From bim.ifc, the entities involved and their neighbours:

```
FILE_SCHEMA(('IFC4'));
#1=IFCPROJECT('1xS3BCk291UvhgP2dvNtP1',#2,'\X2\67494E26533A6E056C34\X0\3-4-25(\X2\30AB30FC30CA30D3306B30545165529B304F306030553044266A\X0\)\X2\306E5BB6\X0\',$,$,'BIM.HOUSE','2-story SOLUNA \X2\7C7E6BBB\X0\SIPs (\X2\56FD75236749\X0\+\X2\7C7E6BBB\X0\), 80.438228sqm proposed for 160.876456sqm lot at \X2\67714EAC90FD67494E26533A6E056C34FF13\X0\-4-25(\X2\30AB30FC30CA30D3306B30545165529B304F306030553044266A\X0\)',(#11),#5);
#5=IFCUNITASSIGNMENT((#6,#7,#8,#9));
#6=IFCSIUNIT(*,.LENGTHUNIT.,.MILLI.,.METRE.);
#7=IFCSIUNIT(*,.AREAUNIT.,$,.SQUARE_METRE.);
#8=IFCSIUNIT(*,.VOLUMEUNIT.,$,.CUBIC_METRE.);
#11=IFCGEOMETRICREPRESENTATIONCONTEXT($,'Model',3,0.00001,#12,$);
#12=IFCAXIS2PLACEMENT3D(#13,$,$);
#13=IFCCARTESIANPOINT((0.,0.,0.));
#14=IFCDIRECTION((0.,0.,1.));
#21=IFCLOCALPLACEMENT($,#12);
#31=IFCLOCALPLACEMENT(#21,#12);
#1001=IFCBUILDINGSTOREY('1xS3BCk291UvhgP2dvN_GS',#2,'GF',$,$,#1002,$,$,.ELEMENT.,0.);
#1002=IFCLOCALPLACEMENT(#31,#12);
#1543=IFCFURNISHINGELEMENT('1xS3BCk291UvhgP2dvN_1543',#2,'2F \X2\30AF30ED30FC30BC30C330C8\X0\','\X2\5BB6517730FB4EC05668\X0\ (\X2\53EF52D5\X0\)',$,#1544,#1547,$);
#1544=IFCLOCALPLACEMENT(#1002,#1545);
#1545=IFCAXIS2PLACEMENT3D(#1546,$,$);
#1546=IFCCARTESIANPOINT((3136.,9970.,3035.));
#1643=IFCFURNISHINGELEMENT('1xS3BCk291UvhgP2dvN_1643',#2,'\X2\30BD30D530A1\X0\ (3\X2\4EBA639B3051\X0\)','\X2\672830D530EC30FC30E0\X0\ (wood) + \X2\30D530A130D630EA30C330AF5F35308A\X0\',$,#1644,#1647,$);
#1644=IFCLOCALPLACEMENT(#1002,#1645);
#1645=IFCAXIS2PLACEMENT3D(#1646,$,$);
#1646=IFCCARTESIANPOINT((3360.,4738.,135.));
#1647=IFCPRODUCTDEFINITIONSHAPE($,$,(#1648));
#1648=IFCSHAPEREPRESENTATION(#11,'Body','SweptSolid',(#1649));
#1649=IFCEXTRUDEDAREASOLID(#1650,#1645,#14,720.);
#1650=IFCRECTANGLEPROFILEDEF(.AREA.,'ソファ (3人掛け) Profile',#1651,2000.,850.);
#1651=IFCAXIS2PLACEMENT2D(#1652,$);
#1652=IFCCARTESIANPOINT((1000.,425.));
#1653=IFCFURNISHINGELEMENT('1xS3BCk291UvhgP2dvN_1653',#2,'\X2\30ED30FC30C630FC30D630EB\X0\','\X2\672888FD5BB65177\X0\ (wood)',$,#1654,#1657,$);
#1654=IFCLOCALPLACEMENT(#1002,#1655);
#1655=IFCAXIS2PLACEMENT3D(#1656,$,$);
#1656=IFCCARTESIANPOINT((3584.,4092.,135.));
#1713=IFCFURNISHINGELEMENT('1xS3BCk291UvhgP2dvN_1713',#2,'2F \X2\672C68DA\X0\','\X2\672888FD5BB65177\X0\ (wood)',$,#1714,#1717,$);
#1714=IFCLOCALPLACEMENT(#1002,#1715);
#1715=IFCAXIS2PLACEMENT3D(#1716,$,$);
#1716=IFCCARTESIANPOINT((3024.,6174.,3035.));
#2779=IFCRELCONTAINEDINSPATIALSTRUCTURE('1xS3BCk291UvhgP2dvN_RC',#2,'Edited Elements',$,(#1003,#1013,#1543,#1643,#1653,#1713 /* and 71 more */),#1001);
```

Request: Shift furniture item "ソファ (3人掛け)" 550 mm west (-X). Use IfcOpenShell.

```python
import ifcopenshell
import ifcopenshell.api.geometry
import ifcopenshell.util.placement
import ifcopenshell.util.unit

model = ifcopenshell.open("bim.ifc")
unit_scale = ifcopenshell.util.unit.calculate_unit_scale(model)

item = model.by_id(1643)
matrix = ifcopenshell.util.placement.get_local_placement(item.ObjectPlacement)
matrix[0, 3] -= 0.55 / unit_scale
ifcopenshell.api.geometry.edit_object_placement(model, product=item, matrix=matrix, is_si=False)

print(ifcopenshell.util.placement.get_local_placement(item.ObjectPlacement).round(3) + 0.0)

model.write("bim_rev.ifc")
```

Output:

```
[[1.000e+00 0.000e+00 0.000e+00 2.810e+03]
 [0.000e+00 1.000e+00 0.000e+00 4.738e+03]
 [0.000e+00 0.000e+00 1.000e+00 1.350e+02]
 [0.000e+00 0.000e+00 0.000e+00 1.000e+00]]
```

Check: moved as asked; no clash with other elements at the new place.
